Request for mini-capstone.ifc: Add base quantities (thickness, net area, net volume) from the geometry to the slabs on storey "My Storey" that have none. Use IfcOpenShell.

First a look at what the model holds.

```python
import ifcopenshell
import ifcopenshell.util.element
import ifcopenshell.util.unit

model = ifcopenshell.open("mini-capstone.ifc")
print(model.schema)
for unit_type in ("LENGTHUNIT", "AREAUNIT", "VOLUMEUNIT"):
    print(unit_type, ifcopenshell.util.unit.calculate_unit_scale(model, unit_type))
storey = next(s for s in model.by_type("IfcBuildingStorey") if s.Name == "My Storey")
slabs = [e for e in ifcopenshell.util.element.get_decomposition(storey) if e.is_a("IfcSlab")]
for e in sorted(slabs, key=lambda e: e.id()):
    print(e.id(), e.is_a(), e.Name, list(ifcopenshell.util.element.get_psets(e, qtos_only=True)), sep=" | ")
```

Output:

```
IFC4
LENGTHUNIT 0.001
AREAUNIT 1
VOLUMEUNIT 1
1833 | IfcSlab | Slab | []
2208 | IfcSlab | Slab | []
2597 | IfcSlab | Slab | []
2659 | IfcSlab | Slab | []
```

```python
import ifcopenshell
import ifcopenshell.api.pset
import ifcopenshell.geom
import ifcopenshell.util.element
import ifcopenshell.util.shape
import ifcopenshell.util.unit

model = ifcopenshell.open("mini-capstone.ifc")
unit_scale = ifcopenshell.util.unit.calculate_unit_scale(model)
area_scale = ifcopenshell.util.unit.calculate_unit_scale(model, "AREAUNIT")
volume_scale = ifcopenshell.util.unit.calculate_unit_scale(model, "VOLUMEUNIT")
settings = ifcopenshell.geom.settings()

storey = next(s for s in model.by_type("IfcBuildingStorey") if s.Name == "My Storey")
slabs = [e for e in ifcopenshell.util.element.get_decomposition(storey) if e.is_a("IfcSlab")]

for e in sorted(slabs, key=lambda e: e.id()):
    if ifcopenshell.util.element.get_psets(e, qtos_only=True, should_inherit=False):
        continue
    # Geometry comes back in metres, in the element's own axes.
    shape = ifcopenshell.geom.create_shape(settings, e)
    values = {
        "Width": ifcopenshell.util.shape.get_z(shape.geometry) / unit_scale,
        "NetArea": ifcopenshell.util.shape.get_footprint_area(shape.geometry) / area_scale,
        "NetVolume": ifcopenshell.util.shape.get_volume(shape.geometry) / volume_scale,
    }
    qto = ifcopenshell.api.pset.add_qto(model, product=e, name="Qto_SlabBaseQuantities")
    ifcopenshell.api.pset.edit_qto(model, qto=qto, properties=values)
    print(e.id(), {k: round(v, 3) for k, v in values.items()})

model.write("mini-capstone_v2.ifc")
```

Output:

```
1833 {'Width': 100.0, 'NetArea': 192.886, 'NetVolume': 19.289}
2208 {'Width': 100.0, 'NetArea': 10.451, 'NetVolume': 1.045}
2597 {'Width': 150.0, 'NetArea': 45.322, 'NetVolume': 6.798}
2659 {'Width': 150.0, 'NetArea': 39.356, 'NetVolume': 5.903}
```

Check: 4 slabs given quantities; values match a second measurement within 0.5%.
